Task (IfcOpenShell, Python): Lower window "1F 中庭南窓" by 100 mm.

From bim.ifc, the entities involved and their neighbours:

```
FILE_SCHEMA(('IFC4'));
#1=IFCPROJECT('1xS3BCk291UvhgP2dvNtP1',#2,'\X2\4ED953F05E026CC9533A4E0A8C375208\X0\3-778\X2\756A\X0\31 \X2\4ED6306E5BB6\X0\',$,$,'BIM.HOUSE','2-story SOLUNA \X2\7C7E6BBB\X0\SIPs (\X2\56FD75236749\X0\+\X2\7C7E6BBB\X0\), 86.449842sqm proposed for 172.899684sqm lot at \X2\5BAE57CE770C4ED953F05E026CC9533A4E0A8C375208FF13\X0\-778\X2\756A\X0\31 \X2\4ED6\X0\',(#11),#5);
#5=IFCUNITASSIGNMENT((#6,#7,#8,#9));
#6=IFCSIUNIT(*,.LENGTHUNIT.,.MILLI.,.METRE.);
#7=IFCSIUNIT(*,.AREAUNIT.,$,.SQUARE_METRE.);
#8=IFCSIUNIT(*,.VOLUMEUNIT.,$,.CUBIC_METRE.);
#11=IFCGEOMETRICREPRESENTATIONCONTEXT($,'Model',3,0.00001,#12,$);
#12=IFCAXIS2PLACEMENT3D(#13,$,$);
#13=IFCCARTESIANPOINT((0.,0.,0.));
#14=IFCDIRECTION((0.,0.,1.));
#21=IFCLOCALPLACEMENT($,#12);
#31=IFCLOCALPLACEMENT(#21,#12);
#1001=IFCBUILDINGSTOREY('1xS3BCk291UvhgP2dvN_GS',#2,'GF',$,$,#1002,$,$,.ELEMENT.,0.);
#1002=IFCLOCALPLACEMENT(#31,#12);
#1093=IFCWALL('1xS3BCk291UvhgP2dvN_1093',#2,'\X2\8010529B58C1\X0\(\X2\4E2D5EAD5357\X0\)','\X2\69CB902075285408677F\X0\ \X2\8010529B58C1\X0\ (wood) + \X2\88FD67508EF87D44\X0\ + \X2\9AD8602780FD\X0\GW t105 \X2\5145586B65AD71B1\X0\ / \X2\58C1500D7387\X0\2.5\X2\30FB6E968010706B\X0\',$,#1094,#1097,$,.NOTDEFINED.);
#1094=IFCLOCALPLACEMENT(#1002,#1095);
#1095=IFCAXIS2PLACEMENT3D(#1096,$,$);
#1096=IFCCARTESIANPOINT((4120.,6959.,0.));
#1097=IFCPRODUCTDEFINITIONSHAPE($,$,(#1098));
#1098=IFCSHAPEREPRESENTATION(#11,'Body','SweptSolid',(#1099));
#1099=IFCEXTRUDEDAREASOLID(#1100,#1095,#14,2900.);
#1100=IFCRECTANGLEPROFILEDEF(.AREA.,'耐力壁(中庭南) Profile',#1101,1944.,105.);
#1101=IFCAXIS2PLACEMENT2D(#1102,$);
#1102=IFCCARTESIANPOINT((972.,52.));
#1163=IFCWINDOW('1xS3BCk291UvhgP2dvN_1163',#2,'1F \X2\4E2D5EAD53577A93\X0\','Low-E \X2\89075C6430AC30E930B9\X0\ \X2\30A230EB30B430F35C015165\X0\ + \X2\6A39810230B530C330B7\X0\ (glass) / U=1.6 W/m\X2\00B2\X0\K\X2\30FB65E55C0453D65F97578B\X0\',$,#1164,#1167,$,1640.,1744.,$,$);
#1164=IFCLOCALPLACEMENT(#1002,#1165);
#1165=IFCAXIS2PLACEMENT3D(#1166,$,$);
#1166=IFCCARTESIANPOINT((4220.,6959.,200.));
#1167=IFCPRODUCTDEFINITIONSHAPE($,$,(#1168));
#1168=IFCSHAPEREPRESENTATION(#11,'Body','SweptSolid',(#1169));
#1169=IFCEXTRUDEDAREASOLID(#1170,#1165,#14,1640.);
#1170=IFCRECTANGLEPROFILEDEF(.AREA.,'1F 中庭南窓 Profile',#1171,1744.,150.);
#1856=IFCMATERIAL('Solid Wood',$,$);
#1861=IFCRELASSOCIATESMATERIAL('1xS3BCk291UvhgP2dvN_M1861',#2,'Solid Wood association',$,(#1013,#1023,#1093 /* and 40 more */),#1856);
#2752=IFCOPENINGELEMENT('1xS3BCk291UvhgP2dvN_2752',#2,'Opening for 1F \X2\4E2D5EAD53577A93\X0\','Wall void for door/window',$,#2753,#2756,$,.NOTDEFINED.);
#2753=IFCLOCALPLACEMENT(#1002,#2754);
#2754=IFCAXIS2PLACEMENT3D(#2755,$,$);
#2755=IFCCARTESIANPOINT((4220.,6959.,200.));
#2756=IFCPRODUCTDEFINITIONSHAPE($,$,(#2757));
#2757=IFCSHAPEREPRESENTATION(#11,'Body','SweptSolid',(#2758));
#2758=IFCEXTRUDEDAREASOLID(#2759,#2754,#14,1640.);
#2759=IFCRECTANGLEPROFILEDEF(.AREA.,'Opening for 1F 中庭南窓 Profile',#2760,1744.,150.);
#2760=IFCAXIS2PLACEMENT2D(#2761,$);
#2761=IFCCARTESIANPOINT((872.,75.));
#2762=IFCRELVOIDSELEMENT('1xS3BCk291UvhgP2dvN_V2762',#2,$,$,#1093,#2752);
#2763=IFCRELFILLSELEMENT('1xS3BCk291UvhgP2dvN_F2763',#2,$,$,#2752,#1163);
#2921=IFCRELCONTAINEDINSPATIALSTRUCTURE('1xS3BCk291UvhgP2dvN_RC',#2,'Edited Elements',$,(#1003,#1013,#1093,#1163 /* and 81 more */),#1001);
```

```python
import numpy as np
import ifcopenshell
import ifcopenshell.api.geometry
import ifcopenshell.util.placement
import ifcopenshell.util.unit

model = ifcopenshell.open("bim.ifc")
unit_scale = ifcopenshell.util.unit.calculate_unit_scale(model)

window = model.by_guid("1xS3BCk291UvhgP2dvN_1163")
opening = window.FillsVoids[0].RelatingOpeningElement
dz = -100.0

shift = np.array([0.0, 0.0, dz])
# The window is not placed relative to its opening, so move both.
for product in (opening, window):
    matrix = ifcopenshell.util.placement.get_local_placement(product.ObjectPlacement)
    matrix[:3, 3] += shift
    ifcopenshell.api.geometry.edit_object_placement(model, product=product, matrix=matrix, is_si=False)

print(f"moved by {dz * unit_scale:+.3f} m")

model.write("bim-out.ifc")
```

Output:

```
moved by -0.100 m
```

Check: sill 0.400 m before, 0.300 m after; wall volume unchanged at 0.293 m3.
